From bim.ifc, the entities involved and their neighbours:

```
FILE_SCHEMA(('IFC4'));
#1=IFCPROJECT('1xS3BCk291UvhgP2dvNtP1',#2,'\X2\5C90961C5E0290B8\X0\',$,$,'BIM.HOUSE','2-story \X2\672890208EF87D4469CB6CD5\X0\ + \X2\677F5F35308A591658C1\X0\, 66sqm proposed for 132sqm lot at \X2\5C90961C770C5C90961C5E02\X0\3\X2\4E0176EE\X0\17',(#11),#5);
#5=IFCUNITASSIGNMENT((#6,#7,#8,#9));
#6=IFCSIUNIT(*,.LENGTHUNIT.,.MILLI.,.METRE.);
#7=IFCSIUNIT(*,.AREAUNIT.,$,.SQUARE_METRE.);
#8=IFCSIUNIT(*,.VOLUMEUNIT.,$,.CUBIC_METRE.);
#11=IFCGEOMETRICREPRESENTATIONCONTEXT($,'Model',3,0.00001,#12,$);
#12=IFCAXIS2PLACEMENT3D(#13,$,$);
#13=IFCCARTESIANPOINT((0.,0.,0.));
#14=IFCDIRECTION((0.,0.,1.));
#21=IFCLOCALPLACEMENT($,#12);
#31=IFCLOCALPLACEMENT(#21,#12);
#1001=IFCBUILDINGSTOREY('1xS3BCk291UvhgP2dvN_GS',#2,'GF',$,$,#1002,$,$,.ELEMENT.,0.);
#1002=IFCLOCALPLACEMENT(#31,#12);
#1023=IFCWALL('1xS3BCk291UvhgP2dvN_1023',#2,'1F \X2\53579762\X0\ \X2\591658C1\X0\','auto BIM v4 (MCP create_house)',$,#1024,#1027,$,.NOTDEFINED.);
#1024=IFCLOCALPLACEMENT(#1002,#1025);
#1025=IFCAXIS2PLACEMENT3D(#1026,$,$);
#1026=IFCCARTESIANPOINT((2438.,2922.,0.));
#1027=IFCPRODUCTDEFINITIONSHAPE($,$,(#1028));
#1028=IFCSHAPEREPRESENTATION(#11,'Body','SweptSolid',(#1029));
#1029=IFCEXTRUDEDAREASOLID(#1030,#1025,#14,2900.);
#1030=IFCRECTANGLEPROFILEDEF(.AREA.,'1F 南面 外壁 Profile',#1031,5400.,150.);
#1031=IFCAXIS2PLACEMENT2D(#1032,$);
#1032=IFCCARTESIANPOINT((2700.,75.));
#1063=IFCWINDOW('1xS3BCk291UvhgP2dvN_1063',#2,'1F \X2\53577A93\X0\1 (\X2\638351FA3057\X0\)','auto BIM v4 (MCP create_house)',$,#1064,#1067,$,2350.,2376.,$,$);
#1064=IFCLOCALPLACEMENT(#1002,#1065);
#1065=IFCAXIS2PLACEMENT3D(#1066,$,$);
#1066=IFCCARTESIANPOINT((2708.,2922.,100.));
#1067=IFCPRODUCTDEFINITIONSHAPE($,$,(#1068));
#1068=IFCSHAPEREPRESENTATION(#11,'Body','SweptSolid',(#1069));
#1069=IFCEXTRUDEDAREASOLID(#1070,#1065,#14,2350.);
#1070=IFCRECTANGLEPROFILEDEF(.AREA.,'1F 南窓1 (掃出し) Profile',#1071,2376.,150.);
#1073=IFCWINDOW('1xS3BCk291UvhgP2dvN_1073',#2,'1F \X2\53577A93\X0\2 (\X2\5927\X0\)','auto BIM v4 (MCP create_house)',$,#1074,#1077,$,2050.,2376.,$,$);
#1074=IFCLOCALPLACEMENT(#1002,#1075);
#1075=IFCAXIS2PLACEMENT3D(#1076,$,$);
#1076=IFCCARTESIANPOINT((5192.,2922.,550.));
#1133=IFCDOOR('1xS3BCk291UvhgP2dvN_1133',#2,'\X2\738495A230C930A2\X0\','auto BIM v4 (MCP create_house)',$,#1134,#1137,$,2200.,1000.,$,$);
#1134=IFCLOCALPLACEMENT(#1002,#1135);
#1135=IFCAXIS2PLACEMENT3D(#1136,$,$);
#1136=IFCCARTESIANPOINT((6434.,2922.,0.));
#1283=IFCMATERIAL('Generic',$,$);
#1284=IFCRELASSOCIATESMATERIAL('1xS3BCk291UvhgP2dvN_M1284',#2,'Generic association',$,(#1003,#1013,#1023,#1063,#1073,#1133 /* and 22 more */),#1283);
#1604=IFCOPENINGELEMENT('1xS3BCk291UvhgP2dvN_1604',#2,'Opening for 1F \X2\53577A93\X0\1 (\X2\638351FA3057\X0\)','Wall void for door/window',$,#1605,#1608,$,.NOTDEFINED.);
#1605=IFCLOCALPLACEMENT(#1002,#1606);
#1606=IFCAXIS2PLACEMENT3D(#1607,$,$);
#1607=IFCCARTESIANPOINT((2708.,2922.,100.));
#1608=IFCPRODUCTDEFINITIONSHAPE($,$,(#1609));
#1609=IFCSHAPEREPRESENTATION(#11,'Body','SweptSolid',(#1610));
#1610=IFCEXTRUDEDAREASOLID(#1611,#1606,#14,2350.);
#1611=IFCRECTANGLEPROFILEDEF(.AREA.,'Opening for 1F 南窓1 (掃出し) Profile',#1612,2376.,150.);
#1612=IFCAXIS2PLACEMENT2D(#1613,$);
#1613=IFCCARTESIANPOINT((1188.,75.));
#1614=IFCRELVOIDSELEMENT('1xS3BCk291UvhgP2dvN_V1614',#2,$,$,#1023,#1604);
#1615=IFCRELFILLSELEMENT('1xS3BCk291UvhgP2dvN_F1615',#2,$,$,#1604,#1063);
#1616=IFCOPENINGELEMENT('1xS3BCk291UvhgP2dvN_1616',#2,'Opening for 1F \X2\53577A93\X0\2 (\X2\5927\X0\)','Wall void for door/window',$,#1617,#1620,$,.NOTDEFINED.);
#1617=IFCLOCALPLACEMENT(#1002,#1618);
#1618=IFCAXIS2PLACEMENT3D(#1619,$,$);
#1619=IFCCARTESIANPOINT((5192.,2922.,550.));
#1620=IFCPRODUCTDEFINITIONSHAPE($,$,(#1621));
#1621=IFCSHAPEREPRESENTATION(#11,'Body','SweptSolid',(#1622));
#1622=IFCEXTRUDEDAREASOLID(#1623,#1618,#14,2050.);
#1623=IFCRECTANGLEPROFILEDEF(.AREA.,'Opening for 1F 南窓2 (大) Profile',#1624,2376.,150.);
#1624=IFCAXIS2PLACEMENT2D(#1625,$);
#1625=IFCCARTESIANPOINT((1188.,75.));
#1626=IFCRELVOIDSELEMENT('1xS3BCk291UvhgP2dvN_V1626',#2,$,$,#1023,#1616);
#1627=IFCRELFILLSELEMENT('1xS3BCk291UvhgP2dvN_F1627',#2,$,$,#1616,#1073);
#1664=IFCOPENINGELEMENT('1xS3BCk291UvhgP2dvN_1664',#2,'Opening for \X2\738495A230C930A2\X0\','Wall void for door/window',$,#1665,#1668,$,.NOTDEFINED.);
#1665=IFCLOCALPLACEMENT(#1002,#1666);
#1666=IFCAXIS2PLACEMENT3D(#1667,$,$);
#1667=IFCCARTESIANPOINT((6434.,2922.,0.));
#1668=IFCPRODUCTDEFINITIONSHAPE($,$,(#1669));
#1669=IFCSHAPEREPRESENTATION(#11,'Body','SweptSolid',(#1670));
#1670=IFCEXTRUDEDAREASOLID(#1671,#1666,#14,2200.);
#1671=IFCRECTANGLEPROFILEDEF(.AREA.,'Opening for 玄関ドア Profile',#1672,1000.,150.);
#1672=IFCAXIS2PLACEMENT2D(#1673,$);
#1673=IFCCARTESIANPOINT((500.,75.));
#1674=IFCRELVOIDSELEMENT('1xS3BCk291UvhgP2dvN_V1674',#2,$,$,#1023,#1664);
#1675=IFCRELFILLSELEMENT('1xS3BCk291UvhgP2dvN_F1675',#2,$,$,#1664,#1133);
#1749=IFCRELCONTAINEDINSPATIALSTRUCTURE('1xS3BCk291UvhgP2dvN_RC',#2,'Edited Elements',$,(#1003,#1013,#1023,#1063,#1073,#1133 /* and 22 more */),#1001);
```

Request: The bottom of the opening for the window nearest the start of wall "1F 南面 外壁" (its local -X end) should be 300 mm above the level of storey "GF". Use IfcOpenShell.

```python
import numpy as np
import ifcopenshell
import ifcopenshell.api.geometry
import ifcopenshell.geom
import ifcopenshell.util.element
import ifcopenshell.util.placement
import ifcopenshell.util.shape
import ifcopenshell.util.unit

model = ifcopenshell.open("bim.ifc")
unit_scale = ifcopenshell.util.unit.calculate_unit_scale(model)

window = model.by_guid("1xS3BCk291UvhgP2dvN_1063")
opening = window.FillsVoids[0].RelatingOpeningElement
storey = ifcopenshell.util.element.get_container(window, ifc_class="IfcBuildingStorey")
level = ifcopenshell.util.placement.get_local_placement(storey.ObjectPlacement)[2, 3]

# The opening's origin need not be at the sill, so measure its lowest point.
shape = ifcopenshell.geom.create_shape(ifcopenshell.geom.settings(), opening)
bottom = ifcopenshell.util.shape.get_shape_bottom_elevation(shape, shape.geometry) / unit_scale
dz = level + 300.0 - bottom

shift = np.array([0.0, 0.0, dz])
# The window is not placed relative to its opening, so move both.
for product in (opening, window):
    matrix = ifcopenshell.util.placement.get_local_placement(product.ObjectPlacement)
    matrix[:3, 3] += shift
    ifcopenshell.api.geometry.edit_object_placement(model, product=product, matrix=matrix, is_si=False)

print(f"moved by {dz * unit_scale:+.3f} m")

model.write("bim-out.ifc")
```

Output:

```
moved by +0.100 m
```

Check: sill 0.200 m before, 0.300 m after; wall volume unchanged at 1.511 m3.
